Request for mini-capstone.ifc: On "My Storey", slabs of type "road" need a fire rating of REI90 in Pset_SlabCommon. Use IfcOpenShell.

First a look at what the model holds.

```python
import ifcopenshell
import ifcopenshell.util.element

model = ifcopenshell.open("mini-capstone.ifc")
print(model.schema)
storey = next(s for s in model.by_type("IfcBuildingStorey") if s.Name == "My Storey")
slabs = [e for e in ifcopenshell.util.element.get_decomposition(storey) if e.is_a("IfcSlab")]
seen = {}
for e in slabs:
    element_type = ifcopenshell.util.element.get_type(e)
    key = (element_type.Name if element_type != e and element_type else None, ifcopenshell.util.element.get_pset(e, "Pset_SlabCommon", "FireRating"))
    seen[key] = seen.get(key, 0) + 1
for (name, value), count in sorted(seen.items(), key=str):
    print(count, "x", name, "|", value)
```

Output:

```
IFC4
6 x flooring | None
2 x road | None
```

```python
import ifcopenshell
import ifcopenshell.api.pset
import ifcopenshell.util.element

model = ifcopenshell.open("mini-capstone.ifc")

storey = next(s for s in model.by_type("IfcBuildingStorey") if s.Name == "My Storey")
slabs = [e for e in ifcopenshell.util.element.get_decomposition(storey) if e.is_a("IfcSlab")]

count = 0
for e in slabs:
    element_type = ifcopenshell.util.element.get_type(e)
    if element_type in (None, e) or element_type.Name != "road":
        continue
    # add_pset returns the element's existing set when there is one.
    pset = ifcopenshell.api.pset.add_pset(model, product=e, name="Pset_SlabCommon")
    ifcopenshell.api.pset.edit_pset(model, pset=pset, properties={"FireRating": "REI90"})
    count += 1

print(count, "slabs updated")

model.write("mini-capstone_updated.ifc")
```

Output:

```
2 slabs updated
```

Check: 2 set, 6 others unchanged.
